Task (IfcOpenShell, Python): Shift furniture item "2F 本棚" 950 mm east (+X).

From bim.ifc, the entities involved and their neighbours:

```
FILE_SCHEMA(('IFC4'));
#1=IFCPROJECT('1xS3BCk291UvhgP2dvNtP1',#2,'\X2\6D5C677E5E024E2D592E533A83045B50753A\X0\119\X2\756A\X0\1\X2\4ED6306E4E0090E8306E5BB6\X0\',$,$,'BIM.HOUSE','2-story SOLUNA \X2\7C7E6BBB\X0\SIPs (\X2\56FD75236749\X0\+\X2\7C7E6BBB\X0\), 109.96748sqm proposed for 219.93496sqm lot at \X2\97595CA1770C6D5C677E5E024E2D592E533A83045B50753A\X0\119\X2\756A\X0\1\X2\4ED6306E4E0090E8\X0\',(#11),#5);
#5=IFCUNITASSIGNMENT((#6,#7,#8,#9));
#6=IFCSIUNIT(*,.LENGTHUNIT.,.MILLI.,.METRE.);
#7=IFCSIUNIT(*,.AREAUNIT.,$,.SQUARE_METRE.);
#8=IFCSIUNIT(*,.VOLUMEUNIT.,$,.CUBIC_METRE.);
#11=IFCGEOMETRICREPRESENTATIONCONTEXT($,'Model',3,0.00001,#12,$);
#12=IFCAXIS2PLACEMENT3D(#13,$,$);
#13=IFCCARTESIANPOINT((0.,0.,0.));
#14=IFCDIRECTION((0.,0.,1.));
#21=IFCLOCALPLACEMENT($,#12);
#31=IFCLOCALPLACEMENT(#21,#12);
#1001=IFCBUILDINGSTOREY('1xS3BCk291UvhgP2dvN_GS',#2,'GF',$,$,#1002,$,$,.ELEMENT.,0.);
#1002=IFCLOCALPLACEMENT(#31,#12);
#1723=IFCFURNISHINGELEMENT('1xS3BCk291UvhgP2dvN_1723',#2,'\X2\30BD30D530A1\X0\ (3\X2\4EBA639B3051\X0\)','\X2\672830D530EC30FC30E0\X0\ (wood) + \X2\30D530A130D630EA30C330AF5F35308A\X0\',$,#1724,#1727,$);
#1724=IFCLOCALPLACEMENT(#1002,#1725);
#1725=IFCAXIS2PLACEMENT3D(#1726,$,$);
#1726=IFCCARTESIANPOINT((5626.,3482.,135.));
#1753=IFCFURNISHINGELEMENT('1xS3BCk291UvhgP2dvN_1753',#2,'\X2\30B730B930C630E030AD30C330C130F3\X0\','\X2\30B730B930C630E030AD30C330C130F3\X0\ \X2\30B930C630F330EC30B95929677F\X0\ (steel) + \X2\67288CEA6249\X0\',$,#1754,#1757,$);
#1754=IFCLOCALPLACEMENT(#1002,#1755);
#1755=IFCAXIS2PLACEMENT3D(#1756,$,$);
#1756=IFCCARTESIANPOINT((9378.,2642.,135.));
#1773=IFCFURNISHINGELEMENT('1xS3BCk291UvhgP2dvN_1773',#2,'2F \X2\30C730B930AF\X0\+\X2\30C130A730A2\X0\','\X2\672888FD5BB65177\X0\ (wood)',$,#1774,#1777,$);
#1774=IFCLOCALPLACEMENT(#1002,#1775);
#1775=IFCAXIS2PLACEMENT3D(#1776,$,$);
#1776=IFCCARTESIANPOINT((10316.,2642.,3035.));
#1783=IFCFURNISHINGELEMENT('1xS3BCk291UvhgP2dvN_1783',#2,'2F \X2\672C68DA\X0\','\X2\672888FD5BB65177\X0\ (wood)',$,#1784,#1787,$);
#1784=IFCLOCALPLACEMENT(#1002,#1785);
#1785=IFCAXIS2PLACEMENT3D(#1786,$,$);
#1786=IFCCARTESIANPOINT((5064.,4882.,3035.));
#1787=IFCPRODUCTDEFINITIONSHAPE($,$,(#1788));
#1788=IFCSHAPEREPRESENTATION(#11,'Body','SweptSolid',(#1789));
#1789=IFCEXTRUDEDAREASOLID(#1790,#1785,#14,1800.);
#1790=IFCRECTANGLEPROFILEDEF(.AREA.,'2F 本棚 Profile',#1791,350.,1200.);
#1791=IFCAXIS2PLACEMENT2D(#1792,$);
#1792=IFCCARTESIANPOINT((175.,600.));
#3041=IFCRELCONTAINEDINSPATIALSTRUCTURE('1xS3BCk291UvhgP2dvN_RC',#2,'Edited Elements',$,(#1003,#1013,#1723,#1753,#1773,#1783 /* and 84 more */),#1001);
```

```python
import ifcopenshell
import ifcopenshell.api.geometry
import ifcopenshell.util.placement

model = ifcopenshell.open("bim.ifc")

item = model.by_guid("1xS3BCk291UvhgP2dvN_1783")
matrix = ifcopenshell.util.placement.get_local_placement(item.ObjectPlacement)
matrix[0, 3] += 950.0
ifcopenshell.api.geometry.edit_object_placement(model, product=item, matrix=matrix, is_si=False)

print(ifcopenshell.util.placement.get_local_placement(item.ObjectPlacement).round(3) + 0.0)

model.write("bim_v2.ifc")
```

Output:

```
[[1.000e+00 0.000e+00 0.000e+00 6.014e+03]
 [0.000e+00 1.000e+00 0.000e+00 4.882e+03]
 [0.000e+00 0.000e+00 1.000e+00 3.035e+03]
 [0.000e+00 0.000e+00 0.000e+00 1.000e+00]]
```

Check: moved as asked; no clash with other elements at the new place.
